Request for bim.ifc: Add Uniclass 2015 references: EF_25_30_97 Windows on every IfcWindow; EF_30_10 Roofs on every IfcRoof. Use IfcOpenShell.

First a look at what the model holds.

```python
import ifcopenshell

model = ifcopenshell.open("bim.ifc")
print(model.schema)
print("classifications:", [c.Name for c in model.by_type("IfcClassification")])
for ifc_class in ("IfcDoor", "IfcRoof", "IfcStair", "IfcWall", "IfcWindow"):
    print(ifc_class, len(model.by_type(ifc_class)))
```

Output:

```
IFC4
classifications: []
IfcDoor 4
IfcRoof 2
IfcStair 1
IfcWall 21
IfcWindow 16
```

```python
import ifcopenshell
import ifcopenshell.api.classification

model = ifcopenshell.open("bim.ifc")

system = ifcopenshell.api.classification.add_classification(model, classification="Uniclass 2015")

codes = {
    "IfcWindow": ("EF_25_30_97", "Windows"),
    "IfcRoof": ("EF_30_10", "Roofs"),
}
for ifc_class, (code, name) in codes.items():
    products = model.by_type(ifc_class)
    ifcopenshell.api.classification.add_reference(
        model, products=products, classification=system, identification=code, name=name
    )
    print(code, len(products))

model.write("bim-out.ifc")
```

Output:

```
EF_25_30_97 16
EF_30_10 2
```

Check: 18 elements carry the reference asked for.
